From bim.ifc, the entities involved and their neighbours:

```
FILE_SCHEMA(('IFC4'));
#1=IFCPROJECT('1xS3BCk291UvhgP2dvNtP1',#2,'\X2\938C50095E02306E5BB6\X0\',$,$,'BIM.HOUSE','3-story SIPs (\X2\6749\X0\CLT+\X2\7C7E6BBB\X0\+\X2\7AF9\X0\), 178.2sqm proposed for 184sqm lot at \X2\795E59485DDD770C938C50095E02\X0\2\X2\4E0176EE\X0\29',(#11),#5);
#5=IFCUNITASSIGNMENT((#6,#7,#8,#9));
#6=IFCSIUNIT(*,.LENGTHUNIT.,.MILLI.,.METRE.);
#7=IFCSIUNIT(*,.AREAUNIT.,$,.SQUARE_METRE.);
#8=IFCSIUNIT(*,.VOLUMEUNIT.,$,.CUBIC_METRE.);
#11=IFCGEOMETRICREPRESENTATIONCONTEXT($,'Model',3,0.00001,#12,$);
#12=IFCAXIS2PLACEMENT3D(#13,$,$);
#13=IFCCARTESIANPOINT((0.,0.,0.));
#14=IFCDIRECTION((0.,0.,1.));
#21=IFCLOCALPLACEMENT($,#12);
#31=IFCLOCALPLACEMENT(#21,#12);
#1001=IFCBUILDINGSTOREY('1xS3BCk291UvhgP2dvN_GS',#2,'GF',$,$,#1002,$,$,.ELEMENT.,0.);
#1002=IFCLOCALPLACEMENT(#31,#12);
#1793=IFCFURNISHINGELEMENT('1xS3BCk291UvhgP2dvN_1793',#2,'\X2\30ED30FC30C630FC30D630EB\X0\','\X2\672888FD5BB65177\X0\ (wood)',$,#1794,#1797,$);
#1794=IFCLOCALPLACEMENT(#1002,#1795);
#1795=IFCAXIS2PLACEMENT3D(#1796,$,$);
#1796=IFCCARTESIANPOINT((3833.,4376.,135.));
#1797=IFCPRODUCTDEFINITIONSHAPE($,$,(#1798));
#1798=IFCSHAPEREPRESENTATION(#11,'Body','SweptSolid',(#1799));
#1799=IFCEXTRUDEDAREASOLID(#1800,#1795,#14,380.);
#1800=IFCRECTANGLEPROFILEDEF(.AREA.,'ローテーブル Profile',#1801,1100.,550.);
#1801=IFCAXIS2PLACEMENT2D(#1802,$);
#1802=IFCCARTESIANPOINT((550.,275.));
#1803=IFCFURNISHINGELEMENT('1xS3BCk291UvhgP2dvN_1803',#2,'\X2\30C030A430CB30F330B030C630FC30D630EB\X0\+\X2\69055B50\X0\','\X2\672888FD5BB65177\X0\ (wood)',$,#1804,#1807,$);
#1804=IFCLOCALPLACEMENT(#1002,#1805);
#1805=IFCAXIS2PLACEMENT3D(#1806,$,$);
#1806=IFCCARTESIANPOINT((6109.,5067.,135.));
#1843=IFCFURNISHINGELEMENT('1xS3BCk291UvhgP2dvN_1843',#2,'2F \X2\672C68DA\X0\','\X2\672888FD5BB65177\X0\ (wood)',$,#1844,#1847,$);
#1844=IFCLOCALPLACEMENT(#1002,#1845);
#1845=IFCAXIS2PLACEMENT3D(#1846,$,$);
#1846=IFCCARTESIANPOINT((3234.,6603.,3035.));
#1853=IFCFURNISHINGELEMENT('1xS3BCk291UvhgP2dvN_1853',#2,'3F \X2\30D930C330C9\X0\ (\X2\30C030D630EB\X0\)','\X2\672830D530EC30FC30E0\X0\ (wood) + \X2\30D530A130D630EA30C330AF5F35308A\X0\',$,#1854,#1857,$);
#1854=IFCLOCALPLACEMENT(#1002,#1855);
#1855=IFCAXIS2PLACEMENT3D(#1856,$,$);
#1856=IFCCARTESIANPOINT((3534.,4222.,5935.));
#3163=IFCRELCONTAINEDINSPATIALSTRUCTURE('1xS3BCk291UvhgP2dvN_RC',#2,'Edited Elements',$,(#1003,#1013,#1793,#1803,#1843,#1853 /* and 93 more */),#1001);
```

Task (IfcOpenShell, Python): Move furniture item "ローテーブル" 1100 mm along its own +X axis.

```python
import ifcopenshell
import ifcopenshell.api.geometry
import ifcopenshell.util.placement
import ifcopenshell.util.unit

model = ifcopenshell.open("bim.ifc")
unit_scale = ifcopenshell.util.unit.calculate_unit_scale(model)

item = model.by_id(1793)
matrix = ifcopenshell.util.placement.get_local_placement(item.ObjectPlacement)
matrix[:3, 3] += matrix[:3, 0] * 1.1 / unit_scale
ifcopenshell.api.geometry.edit_object_placement(model, product=item, matrix=matrix, is_si=False)

print(ifcopenshell.util.placement.get_local_placement(item.ObjectPlacement).round(3) + 0.0)

model.write("bim_v2.ifc")
```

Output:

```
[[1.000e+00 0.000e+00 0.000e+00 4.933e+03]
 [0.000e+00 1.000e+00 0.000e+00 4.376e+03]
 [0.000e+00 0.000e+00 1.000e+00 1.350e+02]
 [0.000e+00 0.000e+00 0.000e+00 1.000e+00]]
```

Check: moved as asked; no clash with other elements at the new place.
